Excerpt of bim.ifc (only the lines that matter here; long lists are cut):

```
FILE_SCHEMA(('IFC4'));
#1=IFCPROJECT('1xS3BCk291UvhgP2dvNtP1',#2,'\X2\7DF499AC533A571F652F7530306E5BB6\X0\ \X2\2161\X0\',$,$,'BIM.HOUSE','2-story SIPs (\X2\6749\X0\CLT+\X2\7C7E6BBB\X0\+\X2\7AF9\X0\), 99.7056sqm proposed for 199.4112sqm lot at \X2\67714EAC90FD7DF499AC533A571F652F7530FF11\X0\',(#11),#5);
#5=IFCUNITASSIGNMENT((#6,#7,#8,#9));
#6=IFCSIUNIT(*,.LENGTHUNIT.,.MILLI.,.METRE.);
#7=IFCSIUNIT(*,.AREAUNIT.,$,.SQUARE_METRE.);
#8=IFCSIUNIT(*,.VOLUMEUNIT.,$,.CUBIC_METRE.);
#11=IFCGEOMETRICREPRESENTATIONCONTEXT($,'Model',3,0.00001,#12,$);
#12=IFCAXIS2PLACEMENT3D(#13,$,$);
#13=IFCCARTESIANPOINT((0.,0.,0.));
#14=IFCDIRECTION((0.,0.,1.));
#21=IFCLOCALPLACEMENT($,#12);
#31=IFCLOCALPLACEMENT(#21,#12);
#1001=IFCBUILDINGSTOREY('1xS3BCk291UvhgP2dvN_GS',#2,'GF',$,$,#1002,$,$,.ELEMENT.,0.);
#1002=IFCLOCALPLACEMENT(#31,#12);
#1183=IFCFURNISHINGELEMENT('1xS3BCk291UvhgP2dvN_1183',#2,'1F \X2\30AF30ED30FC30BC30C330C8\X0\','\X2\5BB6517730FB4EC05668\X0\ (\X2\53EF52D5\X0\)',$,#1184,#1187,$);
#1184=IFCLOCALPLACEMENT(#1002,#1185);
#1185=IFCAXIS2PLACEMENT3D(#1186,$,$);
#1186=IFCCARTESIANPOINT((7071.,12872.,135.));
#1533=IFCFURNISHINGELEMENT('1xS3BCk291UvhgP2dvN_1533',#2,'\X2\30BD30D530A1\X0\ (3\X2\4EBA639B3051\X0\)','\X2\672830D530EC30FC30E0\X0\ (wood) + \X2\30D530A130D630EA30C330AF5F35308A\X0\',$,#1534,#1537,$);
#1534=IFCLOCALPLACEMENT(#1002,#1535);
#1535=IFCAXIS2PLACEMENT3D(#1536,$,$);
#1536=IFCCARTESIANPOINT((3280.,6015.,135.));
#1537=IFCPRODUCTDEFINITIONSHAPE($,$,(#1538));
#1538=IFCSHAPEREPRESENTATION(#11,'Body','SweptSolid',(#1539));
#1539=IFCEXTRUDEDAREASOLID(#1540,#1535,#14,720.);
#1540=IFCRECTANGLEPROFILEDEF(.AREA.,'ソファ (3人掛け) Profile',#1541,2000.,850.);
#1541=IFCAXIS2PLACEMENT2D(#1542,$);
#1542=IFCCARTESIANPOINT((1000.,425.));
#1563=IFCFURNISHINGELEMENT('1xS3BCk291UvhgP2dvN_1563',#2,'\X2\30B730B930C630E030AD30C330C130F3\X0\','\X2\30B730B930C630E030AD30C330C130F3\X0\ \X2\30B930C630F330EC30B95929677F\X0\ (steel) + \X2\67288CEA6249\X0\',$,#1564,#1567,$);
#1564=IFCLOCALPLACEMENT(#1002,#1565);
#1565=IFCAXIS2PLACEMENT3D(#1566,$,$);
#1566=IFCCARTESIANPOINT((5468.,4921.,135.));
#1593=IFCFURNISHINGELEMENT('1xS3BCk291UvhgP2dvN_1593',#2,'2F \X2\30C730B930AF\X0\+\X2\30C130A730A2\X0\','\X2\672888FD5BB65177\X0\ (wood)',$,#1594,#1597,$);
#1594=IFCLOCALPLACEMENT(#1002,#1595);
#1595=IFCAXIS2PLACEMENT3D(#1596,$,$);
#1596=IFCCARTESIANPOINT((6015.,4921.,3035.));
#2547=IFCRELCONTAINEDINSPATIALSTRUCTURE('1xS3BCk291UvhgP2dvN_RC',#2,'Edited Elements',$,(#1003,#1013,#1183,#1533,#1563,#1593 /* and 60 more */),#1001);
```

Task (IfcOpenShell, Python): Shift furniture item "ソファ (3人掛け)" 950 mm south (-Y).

```python
import ifcopenshell
import ifcopenshell.api.geometry
import ifcopenshell.util.placement
import ifcopenshell.util.unit

model = ifcopenshell.open("bim.ifc")
unit_scale = ifcopenshell.util.unit.calculate_unit_scale(model)

item = model.by_guid("1xS3BCk291UvhgP2dvN_1533")
matrix = ifcopenshell.util.placement.get_local_placement(item.ObjectPlacement)
matrix[1, 3] -= 0.95 / unit_scale
ifcopenshell.api.geometry.edit_object_placement(model, product=item, matrix=matrix, is_si=False)

print(ifcopenshell.util.placement.get_local_placement(item.ObjectPlacement).round(3) + 0.0)

model.write("bim_v2.ifc")
```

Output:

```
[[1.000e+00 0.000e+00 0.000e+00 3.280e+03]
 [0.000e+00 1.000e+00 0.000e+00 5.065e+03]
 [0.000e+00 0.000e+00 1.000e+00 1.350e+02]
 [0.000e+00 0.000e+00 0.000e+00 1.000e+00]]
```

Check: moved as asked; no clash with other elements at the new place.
